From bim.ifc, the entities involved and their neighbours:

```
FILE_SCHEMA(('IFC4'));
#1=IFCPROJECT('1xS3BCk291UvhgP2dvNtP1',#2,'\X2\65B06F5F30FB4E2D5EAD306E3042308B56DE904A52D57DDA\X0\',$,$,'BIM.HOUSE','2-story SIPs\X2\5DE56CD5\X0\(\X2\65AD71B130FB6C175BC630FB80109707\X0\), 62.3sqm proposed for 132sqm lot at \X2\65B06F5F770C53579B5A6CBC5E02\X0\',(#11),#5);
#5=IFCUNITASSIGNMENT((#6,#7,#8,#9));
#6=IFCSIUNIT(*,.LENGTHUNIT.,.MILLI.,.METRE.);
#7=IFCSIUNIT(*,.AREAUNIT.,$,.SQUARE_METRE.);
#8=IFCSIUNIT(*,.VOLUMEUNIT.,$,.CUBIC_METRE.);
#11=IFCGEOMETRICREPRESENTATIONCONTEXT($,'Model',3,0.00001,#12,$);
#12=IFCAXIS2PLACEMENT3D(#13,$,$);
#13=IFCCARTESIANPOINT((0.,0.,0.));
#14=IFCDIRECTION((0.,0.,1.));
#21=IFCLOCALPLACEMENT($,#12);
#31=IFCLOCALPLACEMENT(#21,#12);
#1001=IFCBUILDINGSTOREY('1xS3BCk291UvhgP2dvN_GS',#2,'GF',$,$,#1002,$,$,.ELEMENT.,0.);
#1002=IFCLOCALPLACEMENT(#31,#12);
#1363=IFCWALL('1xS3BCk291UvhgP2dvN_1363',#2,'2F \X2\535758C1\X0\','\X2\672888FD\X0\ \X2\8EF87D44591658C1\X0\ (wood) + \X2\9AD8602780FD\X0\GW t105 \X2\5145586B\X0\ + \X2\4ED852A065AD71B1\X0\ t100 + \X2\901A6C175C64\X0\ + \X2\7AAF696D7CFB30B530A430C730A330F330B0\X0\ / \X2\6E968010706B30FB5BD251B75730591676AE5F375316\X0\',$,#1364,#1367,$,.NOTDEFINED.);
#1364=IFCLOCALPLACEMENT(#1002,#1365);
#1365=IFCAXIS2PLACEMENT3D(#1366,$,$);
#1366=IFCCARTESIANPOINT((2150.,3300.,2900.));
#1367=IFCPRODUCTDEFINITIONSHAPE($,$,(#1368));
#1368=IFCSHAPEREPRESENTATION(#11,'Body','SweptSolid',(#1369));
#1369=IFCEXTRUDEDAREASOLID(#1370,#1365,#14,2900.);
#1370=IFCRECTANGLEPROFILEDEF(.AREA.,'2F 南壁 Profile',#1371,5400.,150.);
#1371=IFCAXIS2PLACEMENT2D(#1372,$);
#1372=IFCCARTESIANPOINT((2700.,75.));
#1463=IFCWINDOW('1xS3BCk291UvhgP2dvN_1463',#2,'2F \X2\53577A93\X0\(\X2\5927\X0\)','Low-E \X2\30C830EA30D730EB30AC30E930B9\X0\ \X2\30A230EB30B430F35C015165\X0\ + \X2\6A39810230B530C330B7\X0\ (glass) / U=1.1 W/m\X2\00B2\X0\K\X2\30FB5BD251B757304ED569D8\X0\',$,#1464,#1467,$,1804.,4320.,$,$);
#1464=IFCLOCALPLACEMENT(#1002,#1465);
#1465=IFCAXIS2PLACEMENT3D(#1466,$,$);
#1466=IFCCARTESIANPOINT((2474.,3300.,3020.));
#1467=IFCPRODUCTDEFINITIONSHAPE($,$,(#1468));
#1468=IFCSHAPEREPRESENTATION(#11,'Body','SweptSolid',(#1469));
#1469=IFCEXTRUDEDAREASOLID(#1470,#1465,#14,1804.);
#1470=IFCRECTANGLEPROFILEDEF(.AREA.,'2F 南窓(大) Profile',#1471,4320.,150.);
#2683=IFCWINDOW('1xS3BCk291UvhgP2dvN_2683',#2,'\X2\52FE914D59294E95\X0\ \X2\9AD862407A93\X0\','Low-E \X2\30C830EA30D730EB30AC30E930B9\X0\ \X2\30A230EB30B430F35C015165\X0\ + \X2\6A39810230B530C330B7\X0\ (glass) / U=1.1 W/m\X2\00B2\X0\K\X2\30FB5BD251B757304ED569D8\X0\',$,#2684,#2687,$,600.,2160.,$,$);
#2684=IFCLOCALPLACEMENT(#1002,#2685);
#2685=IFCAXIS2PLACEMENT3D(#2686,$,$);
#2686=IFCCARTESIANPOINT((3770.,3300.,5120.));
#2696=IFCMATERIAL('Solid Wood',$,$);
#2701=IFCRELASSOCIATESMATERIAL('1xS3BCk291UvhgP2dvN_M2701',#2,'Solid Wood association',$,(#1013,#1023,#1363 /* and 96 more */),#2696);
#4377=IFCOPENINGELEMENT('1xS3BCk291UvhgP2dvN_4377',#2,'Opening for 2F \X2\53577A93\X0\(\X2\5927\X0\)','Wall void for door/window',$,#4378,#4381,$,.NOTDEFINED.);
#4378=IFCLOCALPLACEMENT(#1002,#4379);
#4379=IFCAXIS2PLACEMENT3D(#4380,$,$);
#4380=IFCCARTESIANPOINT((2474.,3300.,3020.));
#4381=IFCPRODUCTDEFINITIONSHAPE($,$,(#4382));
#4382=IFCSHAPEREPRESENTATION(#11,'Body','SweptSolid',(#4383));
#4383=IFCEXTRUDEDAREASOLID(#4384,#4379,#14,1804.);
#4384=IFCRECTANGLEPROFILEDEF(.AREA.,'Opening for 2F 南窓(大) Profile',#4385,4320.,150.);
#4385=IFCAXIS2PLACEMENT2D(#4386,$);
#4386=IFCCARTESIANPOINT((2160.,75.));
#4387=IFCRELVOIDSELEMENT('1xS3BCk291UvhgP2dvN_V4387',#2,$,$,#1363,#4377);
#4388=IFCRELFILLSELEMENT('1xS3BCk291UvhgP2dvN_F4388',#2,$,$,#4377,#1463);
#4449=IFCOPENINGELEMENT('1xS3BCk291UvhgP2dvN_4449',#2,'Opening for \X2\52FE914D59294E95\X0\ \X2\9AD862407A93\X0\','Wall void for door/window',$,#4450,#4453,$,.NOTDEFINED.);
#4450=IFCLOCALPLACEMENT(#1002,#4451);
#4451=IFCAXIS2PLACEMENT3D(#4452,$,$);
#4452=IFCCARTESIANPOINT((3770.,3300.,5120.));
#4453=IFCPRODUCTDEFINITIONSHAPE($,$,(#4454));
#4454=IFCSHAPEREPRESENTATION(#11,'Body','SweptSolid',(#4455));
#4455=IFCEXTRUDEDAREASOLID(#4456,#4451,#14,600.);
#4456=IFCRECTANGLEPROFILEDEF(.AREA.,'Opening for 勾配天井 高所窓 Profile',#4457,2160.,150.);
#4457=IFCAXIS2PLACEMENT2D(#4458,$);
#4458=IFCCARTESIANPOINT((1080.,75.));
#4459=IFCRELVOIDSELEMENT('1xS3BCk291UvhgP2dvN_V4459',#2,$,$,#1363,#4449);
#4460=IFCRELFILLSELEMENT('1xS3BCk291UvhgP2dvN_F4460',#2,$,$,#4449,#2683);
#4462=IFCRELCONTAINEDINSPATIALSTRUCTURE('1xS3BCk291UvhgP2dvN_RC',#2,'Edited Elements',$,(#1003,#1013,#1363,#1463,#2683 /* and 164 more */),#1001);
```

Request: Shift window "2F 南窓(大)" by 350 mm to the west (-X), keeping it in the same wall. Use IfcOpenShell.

```python
import ifcopenshell
import ifcopenshell.api.geometry
import ifcopenshell.util.placement
import ifcopenshell.util.unit

model = ifcopenshell.open("bim.ifc")
unit_scale = ifcopenshell.util.unit.calculate_unit_scale(model)

window = model.by_guid("1xS3BCk291UvhgP2dvN_1463")
opening = window.FillsVoids[0].RelatingOpeningElement
wall = opening.VoidsElements[0].RelatingBuildingElement

wall_matrix = ifcopenshell.util.placement.get_local_placement(wall.ObjectPlacement)
shift = wall_matrix[:3, 0] * -0.35 / unit_scale
before = ifcopenshell.util.placement.get_local_placement(window.ObjectPlacement)[:3, 3].copy()

# The window is not placed relative to its opening, so move both.
for product in (opening, window):
    matrix = ifcopenshell.util.placement.get_local_placement(product.ObjectPlacement)
    matrix[:3, 3] += shift
    ifcopenshell.api.geometry.edit_object_placement(model, product=product, matrix=matrix, is_si=False)

after = ifcopenshell.util.placement.get_local_placement(window.ObjectPlacement)[:3, 3]
print("window moved by", (after - before).round(3) + 0.0)

model.write("bim_edited.ifc")
```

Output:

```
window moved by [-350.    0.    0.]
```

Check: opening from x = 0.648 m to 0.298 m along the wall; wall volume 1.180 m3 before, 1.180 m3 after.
